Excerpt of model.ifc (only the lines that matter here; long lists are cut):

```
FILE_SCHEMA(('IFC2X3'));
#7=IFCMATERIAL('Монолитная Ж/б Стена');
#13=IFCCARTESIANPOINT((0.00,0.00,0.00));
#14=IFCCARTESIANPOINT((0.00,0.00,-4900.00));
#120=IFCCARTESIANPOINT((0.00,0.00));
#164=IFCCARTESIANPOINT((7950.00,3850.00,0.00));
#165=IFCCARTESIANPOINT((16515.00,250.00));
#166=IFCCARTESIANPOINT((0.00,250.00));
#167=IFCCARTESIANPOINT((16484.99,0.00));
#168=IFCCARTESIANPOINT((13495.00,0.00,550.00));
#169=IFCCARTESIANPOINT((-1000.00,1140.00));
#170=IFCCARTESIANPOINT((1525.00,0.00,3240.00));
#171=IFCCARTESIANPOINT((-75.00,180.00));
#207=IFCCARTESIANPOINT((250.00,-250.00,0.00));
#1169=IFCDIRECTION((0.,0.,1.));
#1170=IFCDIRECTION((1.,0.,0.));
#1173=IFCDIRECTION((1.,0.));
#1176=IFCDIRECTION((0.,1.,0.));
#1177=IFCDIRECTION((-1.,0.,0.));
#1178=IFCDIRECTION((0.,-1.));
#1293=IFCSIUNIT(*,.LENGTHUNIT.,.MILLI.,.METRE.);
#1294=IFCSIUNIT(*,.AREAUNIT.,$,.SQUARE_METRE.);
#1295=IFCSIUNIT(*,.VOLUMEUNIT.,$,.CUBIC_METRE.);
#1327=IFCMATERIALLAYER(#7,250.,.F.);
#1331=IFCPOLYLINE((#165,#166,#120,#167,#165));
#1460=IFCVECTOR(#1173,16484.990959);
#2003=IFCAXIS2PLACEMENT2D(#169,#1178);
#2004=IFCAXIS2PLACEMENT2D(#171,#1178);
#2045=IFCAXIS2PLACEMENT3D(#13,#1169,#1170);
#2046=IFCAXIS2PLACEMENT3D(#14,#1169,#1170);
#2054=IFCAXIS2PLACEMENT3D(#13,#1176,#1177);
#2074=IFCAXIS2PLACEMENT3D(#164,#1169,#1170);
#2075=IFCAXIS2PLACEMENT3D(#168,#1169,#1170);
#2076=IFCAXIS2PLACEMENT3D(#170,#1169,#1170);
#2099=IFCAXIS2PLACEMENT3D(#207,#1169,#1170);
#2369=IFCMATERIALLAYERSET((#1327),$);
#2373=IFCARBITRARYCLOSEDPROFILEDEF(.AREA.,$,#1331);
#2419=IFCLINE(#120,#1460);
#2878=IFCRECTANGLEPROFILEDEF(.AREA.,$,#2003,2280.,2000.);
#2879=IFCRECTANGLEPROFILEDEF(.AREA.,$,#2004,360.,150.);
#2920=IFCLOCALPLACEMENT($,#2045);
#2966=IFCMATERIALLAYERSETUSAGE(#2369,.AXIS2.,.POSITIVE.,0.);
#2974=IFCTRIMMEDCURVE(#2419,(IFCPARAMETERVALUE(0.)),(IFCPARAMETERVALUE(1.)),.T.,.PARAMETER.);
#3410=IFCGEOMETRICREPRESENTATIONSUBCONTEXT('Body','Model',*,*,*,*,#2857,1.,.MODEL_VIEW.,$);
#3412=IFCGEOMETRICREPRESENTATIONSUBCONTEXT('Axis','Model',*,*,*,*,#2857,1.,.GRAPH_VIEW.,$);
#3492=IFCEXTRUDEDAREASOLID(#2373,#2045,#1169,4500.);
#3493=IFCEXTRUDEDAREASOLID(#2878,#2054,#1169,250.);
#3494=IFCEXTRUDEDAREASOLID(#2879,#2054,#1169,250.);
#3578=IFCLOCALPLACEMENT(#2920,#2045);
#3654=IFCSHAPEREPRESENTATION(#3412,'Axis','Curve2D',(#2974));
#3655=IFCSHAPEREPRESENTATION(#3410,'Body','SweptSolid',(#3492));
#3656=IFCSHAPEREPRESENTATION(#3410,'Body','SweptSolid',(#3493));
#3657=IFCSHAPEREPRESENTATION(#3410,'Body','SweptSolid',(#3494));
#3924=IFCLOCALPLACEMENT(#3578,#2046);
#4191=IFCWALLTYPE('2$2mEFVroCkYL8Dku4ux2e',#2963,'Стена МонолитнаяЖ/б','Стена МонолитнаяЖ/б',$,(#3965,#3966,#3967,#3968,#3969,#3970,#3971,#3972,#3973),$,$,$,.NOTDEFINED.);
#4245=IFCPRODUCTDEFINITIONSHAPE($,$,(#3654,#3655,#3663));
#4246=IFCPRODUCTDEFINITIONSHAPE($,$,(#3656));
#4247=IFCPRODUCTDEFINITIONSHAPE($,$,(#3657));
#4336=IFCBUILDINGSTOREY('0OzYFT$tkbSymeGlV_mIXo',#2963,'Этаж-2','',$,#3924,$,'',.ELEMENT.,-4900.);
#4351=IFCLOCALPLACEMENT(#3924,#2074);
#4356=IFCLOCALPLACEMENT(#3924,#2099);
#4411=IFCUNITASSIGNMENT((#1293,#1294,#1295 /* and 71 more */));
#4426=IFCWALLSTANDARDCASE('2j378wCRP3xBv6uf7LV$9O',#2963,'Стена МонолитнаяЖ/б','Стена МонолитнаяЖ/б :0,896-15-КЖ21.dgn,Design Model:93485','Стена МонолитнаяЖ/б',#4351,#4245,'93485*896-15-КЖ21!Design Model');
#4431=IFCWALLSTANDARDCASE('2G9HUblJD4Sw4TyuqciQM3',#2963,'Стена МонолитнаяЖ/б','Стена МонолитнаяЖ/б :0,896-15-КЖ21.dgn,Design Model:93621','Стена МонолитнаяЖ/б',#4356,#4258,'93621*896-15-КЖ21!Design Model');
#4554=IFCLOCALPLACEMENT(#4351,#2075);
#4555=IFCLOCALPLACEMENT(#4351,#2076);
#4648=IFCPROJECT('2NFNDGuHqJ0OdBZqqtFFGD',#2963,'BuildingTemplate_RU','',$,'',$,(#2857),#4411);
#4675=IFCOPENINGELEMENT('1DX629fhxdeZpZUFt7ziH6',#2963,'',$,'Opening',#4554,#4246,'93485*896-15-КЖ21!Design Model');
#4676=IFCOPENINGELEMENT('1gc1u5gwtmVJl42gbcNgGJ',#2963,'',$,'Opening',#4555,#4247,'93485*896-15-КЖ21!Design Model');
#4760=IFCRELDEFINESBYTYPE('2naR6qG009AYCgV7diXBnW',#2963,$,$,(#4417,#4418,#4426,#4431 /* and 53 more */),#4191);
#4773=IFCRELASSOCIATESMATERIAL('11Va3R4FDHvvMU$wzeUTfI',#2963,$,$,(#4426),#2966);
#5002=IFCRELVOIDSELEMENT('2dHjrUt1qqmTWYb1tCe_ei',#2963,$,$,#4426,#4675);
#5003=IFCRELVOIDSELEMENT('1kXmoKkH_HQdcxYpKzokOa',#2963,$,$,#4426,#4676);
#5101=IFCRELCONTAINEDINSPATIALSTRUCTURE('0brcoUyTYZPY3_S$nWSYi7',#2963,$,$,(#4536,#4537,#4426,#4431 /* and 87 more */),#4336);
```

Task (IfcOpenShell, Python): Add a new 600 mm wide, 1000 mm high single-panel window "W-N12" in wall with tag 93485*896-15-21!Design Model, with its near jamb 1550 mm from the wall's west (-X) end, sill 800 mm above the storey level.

```python
import numpy as np
import ifcopenshell
import ifcopenshell.api.feature
import ifcopenshell.api.geometry
import ifcopenshell.api.root
import ifcopenshell.api.spatial
import ifcopenshell.api.type
import ifcopenshell.geom
import ifcopenshell.util.element
import ifcopenshell.util.placement
import ifcopenshell.util.representation
import ifcopenshell.util.shape
import ifcopenshell.util.unit

model = ifcopenshell.open("model.ifc")
unit_scale = ifcopenshell.util.unit.calculate_unit_scale(model)
settings = ifcopenshell.geom.settings()


def volume(element):
    """Net volume in cubic metres, openings subtracted."""
    shape = ifcopenshell.geom.create_shape(settings, element)
    return ifcopenshell.util.shape.get_volume(shape.geometry)


wall = model.by_guid("2j378wCRP3xBv6uf7LV$9O")
storey = ifcopenshell.util.element.get_container(wall, ifc_class="IfcBuildingStorey")
context = ifcopenshell.util.representation.get_context(model, "Model", "Body", "MODEL_VIEW")
before = volume(wall)

width, height, from_end, sill = 0.6, 1, 1.55, 0.8  # metres

# The wall runs along its own X axis, and the end named is its -X end.
wall_shape = ifcopenshell.geom.create_shape(settings, wall)
x, y, z = ifcopenshell.util.shape.get_vertices(wall_shape.geometry).T
start = x.min() + from_end
face, thickness = float(y.min()), float(y.max() - y.min())
wall_matrix = ifcopenshell.util.placement.get_local_placement(wall.ObjectPlacement)
level = ifcopenshell.util.placement.get_local_placement(storey.ObjectPlacement)[2, 3]


def in_wall(x, y):
    """Placement at x, y metres in the wall's axes, at sill height."""
    matrix = wall_matrix.copy()
    matrix[:, 3] = wall_matrix @ np.array([x / unit_scale, y / unit_scale, 0.0, 1.0])
    matrix[2, 3] = level + sill / unit_scale
    return matrix


# Opening: a box that overshoots both wall faces by 50 mm.
opening = ifcopenshell.api.root.create_entity(model, ifc_class="IfcOpeningElement")
box = ifcopenshell.api.geometry.add_wall_representation(
    model, context=context, length=width, height=height, thickness=thickness + 0.1
)
ifcopenshell.api.geometry.assign_representation(model, product=opening, representation=box)
ifcopenshell.api.geometry.edit_object_placement(model, product=opening, matrix=in_wall(start, face - 0.05), is_si=False)
ifcopenshell.api.feature.add_feature(model, feature=opening, element=wall)

window = ifcopenshell.api.root.create_entity(model, ifc_class="IfcWindow", name="W-N12")
window.OverallWidth, window.OverallHeight = width / unit_scale, height / unit_scale
body = ifcopenshell.api.geometry.add_window_representation(
    model,
    context=context,
    overall_width=window.OverallWidth,
    overall_height=window.OverallHeight,
    partition_type="SINGLE_PANEL",
)
ifcopenshell.api.geometry.assign_representation(model, product=window, representation=body)
ifcopenshell.api.spatial.assign_container(model, products=[window], relating_structure=storey)
fills = ifcopenshell.api.feature.add_filling(model, opening=opening, element=window)
fills.OwnerHistory = window.OwnerHistory  # required in IFC2X3

# IFC2X3 keeps the operation on the window style.
style = ifcopenshell.api.root.create_entity(model, ifc_class="IfcWindowStyle", name="W-N12")
style.OperationType, style.ConstructionType = "SINGLE_PANEL", "NOTDEFINED"
style.ParameterTakesPrecedence = style.Sizeable = False
ifcopenshell.api.type.assign_type(model, related_objects=[window], relating_type=style)

# Centre the window in the wall's thickness.
ifcopenshell.api.geometry.edit_object_placement(model, product=window, matrix=in_wall(start, face), is_si=False)
window_shape = ifcopenshell.geom.create_shape(settings, window)
depth = ifcopenshell.util.shape.get_vertices(window_shape.geometry)[:, 1]
offset = face + thickness / 2 - (depth.min() + depth.max()) / 2
ifcopenshell.api.geometry.edit_object_placement(model, product=window, matrix=in_wall(start, offset), is_si=False)

after = volume(wall)

print(f"wall volume {before:.3f} -> {after:.3f} m3")

model.write("model_updated.ifc")
```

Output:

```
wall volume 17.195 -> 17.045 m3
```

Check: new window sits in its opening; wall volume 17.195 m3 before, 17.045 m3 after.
